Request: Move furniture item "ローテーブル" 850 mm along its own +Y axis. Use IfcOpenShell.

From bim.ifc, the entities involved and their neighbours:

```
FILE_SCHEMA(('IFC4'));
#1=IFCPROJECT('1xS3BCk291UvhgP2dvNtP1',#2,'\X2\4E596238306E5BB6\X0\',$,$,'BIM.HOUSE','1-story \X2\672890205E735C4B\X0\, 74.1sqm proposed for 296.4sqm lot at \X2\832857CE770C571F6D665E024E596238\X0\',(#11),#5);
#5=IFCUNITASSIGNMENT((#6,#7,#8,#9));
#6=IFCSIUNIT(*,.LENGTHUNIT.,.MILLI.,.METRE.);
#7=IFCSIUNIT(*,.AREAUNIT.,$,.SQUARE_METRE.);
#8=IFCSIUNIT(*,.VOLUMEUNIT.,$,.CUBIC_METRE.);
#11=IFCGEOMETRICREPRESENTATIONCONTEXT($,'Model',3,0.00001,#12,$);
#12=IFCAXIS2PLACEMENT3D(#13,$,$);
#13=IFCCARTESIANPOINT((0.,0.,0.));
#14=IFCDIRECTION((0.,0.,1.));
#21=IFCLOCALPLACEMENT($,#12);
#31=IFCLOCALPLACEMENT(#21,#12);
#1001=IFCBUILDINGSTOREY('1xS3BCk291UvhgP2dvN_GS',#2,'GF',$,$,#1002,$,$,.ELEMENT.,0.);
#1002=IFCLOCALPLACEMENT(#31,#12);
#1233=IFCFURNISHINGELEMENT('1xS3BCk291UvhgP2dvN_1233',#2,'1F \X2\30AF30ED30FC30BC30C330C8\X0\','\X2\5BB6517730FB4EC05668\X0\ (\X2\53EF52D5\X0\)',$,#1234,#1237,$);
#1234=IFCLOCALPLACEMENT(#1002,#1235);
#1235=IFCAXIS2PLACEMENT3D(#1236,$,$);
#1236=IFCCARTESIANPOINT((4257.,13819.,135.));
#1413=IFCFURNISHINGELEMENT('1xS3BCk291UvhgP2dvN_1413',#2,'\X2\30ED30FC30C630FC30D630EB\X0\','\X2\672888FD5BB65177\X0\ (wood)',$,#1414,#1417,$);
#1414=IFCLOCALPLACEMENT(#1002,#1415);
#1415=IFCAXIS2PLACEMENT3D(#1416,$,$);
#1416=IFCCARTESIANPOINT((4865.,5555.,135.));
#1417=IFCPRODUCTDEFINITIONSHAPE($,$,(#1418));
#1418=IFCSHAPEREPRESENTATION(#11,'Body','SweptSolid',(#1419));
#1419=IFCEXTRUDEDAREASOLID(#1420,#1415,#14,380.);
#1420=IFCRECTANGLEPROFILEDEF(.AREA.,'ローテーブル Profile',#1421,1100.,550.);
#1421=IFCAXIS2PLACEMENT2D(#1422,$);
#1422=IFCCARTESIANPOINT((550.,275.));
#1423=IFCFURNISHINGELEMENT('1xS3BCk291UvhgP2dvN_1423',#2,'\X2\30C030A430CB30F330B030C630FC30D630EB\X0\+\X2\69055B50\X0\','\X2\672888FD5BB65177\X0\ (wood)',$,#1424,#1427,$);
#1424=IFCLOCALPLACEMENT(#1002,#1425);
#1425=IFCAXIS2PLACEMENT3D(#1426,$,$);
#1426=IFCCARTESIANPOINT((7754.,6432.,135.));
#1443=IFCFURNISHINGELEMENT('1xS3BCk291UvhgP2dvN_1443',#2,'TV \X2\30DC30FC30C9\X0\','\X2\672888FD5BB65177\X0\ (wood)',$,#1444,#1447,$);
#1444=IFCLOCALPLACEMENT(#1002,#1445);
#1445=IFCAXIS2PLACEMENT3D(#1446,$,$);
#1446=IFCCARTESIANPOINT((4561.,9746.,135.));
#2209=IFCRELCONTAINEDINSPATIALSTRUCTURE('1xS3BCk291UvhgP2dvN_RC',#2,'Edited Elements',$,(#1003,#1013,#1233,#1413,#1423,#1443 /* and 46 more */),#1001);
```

```python
import ifcopenshell
import ifcopenshell.api.geometry
import ifcopenshell.util.placement
import ifcopenshell.util.unit

model = ifcopenshell.open("bim.ifc")
unit_scale = ifcopenshell.util.unit.calculate_unit_scale(model)

item = model.by_id(1413)
matrix = ifcopenshell.util.placement.get_local_placement(item.ObjectPlacement)
matrix[:3, 3] += matrix[:3, 1] * 0.85 / unit_scale
ifcopenshell.api.geometry.edit_object_placement(model, product=item, matrix=matrix, is_si=False)

print(ifcopenshell.util.placement.get_local_placement(item.ObjectPlacement).round(3) + 0.0)

model.write("bim_edited.ifc")
```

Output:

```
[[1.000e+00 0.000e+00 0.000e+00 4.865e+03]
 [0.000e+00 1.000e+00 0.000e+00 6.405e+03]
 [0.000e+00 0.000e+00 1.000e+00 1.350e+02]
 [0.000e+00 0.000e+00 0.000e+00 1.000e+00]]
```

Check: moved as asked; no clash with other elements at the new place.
